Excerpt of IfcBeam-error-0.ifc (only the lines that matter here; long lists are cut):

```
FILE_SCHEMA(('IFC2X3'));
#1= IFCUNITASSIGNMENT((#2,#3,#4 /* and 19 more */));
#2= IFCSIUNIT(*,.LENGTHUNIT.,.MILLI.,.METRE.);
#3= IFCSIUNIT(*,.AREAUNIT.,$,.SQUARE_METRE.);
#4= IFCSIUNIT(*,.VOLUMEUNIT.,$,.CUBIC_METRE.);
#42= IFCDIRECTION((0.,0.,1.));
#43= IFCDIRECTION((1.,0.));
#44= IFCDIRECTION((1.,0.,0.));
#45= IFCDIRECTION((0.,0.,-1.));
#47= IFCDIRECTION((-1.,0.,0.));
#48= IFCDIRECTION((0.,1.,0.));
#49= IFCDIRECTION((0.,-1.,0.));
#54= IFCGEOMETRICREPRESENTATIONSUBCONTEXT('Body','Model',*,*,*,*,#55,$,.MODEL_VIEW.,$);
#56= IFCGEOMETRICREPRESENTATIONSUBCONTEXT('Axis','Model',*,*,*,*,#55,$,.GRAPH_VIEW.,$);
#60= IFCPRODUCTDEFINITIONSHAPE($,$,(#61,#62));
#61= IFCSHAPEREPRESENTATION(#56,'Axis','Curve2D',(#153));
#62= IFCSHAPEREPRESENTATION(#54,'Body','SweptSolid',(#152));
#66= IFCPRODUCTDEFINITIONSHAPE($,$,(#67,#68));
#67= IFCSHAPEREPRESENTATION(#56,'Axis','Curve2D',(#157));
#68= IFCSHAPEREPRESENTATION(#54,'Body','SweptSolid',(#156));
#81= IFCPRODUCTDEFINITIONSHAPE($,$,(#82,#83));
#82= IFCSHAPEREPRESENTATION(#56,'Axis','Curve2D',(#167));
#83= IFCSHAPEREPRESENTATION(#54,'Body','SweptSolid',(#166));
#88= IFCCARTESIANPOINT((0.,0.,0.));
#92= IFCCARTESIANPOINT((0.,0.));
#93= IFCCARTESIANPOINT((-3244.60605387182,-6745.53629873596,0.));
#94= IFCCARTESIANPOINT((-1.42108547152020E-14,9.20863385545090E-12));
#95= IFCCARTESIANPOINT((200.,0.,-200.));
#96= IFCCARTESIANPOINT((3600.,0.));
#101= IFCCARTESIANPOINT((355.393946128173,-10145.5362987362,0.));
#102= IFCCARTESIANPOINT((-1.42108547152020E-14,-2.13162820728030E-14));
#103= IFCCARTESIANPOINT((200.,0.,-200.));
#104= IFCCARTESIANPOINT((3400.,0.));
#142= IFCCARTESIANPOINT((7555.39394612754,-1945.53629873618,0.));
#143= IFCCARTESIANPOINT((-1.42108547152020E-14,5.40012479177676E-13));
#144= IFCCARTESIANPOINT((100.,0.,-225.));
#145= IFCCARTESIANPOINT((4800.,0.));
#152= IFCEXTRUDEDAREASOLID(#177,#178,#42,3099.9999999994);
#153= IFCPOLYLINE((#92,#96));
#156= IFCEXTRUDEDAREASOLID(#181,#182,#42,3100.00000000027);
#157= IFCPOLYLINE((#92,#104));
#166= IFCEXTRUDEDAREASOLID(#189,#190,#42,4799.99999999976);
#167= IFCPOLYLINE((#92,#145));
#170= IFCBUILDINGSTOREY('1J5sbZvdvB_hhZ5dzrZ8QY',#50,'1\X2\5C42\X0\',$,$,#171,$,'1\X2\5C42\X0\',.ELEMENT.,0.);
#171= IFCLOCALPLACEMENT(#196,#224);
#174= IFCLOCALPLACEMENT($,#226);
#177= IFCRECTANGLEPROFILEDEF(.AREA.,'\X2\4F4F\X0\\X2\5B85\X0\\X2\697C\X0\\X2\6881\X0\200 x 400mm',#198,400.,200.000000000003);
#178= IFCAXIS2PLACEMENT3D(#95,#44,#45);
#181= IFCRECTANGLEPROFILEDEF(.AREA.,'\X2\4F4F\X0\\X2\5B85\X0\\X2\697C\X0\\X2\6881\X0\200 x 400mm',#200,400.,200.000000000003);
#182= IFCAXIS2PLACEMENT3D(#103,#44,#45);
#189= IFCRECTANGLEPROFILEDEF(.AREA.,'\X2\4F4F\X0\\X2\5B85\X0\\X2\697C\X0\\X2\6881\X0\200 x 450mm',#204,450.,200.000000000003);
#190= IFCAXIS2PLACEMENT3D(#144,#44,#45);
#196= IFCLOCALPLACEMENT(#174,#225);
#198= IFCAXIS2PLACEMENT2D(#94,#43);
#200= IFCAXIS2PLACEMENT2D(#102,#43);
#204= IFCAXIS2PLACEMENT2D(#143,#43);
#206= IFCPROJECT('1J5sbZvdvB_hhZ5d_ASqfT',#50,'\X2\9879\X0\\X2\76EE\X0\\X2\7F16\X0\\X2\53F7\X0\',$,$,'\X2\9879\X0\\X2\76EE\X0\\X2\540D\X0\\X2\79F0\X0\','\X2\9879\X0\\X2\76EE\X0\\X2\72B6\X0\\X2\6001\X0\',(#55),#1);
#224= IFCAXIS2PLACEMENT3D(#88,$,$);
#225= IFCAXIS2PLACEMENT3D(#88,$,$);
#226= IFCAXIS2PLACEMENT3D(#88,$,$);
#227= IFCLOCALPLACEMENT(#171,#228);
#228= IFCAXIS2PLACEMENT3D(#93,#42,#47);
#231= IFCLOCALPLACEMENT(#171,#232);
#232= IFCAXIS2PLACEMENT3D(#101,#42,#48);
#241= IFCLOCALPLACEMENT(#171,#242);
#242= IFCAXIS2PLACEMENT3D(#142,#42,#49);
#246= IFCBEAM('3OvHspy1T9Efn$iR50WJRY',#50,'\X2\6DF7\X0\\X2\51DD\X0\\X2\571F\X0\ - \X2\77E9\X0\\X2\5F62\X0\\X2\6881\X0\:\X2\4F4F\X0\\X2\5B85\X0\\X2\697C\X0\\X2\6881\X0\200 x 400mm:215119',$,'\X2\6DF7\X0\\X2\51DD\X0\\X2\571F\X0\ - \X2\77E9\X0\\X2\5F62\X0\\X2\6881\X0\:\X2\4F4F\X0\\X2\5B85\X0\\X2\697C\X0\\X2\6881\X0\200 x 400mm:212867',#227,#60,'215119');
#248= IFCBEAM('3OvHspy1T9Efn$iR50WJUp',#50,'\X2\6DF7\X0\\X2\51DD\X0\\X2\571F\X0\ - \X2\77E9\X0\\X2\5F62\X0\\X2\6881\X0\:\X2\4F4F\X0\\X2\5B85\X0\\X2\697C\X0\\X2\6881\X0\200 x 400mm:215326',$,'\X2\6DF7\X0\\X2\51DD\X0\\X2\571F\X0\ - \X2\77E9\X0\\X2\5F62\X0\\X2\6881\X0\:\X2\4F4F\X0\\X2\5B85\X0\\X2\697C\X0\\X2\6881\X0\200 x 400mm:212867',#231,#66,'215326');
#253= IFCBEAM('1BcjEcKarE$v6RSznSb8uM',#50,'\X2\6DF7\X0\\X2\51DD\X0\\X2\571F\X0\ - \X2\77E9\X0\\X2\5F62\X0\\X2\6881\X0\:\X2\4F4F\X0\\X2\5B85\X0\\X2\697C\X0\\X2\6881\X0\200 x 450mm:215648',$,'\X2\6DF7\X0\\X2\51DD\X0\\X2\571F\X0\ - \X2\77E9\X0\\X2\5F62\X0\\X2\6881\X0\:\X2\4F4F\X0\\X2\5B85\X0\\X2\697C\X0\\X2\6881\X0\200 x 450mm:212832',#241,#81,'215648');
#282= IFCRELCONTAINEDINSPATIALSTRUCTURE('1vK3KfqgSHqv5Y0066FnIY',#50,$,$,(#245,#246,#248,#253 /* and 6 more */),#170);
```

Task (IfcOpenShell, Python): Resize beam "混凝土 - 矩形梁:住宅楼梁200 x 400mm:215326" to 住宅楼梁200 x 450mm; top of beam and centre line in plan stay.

```python
import ifcopenshell
import ifcopenshell.util.element
import ifcopenshell.util.representation

model = ifcopenshell.open("IfcBeam-error-0.ifc")

member = model.by_guid("3OvHspy1T9Efn$iR50WJUp")
source = next(p for p in model.by_type("IfcRectangleProfileDef") if p.ProfileName == "住宅楼梁200 x 450mm")

body = ifcopenshell.util.representation.get_representation(member, "Model", "Body")
solid = body.Items[0]
old_profile = solid.SweptArea

# Copy the section's sizes but keep this member's own profile position.
profile = ifcopenshell.util.element.copy(model, source)
# Profiles are centred, so shift by half the change in depth to hold the top.
shift = (old_profile.XDim - profile.XDim) / 2
x, y = old_profile.Position.Location.Coordinates
up = (-1.0, 0.0)  # upwards, in the solid's own plane
location = model.createIfcCartesianPoint((x + up[0] * shift, y + up[1] * shift))
profile.Position = model.createIfcAxis2Placement2D(location, old_profile.Position.RefDirection)
solid.SweptArea = profile
if not model.get_total_inverses(old_profile):
    ifcopenshell.util.element.remove_deep2(model, old_profile)
member.Name = member.Name.replace("住宅楼梁200 x 400mm", "住宅楼梁200 x 450mm")
member.ObjectType = member.ObjectType.replace("住宅楼梁200 x 400mm", "住宅楼梁200 x 450mm")

print(solid.SweptArea)

model.write("IfcBeam-error-0_v2.ifc")
```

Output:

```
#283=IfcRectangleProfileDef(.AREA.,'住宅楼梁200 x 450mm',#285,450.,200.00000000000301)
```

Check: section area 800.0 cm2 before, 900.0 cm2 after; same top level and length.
